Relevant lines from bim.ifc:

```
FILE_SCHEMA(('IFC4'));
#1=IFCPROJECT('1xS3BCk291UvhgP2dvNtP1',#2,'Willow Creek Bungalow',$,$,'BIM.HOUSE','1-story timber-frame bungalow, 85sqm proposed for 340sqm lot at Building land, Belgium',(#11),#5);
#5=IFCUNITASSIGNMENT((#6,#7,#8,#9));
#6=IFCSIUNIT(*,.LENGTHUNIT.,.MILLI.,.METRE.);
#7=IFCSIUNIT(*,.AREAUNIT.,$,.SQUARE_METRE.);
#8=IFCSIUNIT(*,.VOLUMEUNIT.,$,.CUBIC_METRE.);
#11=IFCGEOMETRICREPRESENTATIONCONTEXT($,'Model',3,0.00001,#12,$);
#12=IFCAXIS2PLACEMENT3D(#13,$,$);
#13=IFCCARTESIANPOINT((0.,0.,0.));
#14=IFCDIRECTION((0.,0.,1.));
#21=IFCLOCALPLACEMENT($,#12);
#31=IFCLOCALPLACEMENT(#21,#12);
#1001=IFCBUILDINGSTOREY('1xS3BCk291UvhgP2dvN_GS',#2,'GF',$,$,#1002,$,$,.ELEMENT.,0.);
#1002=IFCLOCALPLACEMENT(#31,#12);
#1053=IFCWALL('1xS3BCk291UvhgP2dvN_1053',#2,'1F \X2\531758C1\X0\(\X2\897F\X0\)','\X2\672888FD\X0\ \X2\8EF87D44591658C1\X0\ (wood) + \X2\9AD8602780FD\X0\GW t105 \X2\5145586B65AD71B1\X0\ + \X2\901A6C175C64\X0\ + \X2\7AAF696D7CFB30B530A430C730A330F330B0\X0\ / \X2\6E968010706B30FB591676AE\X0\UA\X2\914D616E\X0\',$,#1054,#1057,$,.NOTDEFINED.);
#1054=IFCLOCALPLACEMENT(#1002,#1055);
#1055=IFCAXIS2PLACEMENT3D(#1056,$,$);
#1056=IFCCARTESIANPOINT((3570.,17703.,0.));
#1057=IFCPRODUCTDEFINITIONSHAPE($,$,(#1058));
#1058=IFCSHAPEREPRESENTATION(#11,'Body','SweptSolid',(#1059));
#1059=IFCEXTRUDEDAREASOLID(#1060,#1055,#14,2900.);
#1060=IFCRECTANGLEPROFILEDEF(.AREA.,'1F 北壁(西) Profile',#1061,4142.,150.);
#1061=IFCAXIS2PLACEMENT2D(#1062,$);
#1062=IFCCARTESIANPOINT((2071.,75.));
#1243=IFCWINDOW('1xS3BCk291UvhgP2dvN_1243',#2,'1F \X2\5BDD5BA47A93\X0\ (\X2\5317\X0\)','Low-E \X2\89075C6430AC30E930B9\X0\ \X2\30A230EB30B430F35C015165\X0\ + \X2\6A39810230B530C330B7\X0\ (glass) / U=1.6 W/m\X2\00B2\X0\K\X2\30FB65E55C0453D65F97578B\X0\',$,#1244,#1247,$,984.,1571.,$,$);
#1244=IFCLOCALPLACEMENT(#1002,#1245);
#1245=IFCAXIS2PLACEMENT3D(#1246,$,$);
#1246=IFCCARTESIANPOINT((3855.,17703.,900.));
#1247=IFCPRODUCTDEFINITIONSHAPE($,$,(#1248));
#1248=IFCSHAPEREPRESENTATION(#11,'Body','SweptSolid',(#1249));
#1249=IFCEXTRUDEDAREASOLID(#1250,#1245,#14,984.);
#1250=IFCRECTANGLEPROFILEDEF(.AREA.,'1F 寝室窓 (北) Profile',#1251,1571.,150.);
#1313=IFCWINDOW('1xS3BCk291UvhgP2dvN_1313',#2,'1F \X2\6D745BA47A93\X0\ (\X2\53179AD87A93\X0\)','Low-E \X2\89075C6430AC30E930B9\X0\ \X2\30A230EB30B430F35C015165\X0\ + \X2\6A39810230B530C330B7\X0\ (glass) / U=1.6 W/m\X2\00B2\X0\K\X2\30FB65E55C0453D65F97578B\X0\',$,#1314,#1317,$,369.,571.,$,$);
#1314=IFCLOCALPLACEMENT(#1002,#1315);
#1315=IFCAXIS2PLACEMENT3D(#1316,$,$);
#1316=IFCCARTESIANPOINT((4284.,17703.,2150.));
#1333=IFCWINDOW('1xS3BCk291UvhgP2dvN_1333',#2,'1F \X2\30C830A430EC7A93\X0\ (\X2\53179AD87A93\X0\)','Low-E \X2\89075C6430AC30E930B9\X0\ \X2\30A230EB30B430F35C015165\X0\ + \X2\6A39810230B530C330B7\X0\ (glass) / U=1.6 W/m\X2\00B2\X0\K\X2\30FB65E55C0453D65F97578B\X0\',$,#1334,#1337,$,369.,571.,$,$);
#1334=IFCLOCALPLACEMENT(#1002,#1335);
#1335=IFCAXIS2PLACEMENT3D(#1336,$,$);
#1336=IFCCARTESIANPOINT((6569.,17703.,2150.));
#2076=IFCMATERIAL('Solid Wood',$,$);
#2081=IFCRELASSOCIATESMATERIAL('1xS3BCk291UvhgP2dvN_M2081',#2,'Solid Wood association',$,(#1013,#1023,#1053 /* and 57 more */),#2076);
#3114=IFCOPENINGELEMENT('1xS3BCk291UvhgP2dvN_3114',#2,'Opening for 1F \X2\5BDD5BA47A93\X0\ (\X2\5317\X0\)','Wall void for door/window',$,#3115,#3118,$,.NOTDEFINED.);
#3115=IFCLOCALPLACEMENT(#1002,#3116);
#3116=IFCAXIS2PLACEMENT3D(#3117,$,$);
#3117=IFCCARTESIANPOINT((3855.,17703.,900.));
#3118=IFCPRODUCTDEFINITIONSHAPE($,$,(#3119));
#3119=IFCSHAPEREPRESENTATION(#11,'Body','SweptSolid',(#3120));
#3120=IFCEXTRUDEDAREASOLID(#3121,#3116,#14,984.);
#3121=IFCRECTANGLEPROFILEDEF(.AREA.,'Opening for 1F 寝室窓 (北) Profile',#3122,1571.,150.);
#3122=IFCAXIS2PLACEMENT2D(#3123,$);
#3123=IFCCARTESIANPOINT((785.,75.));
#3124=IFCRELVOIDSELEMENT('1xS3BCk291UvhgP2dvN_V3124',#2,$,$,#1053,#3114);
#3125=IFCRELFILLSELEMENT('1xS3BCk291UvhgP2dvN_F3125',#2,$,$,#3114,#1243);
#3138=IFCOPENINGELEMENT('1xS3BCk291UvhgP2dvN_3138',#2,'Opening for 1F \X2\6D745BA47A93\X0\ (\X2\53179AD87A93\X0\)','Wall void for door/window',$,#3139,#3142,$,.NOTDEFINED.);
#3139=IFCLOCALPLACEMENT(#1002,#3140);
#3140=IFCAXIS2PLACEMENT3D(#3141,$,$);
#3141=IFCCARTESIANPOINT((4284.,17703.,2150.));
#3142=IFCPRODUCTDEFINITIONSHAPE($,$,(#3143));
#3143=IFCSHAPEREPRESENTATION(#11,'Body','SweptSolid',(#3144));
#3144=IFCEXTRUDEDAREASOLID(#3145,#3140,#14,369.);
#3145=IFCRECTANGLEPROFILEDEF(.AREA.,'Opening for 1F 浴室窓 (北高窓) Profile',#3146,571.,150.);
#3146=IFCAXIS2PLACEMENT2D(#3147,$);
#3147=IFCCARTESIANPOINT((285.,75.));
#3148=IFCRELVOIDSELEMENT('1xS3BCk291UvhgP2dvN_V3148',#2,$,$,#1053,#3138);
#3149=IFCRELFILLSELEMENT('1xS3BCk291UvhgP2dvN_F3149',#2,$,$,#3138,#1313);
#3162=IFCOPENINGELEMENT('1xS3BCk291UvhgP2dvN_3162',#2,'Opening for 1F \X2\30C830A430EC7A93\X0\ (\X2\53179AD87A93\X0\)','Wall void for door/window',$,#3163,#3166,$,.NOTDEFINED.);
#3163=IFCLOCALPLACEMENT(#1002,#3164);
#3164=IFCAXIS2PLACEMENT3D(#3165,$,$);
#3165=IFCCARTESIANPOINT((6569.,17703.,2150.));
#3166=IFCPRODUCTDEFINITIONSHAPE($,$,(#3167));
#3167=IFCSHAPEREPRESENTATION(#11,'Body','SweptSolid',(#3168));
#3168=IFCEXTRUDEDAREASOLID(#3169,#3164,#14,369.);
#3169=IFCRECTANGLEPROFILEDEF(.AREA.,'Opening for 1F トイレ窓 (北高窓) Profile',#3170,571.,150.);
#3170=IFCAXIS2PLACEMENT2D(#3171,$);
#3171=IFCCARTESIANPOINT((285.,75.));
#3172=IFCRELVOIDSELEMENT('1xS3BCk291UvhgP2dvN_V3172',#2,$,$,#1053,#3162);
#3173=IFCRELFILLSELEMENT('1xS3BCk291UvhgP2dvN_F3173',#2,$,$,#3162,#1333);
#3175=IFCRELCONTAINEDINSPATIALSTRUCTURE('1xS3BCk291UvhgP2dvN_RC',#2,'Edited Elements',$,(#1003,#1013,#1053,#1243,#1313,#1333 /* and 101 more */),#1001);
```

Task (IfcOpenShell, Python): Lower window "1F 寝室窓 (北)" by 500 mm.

```python
import numpy as np
import ifcopenshell
import ifcopenshell.api.geometry
import ifcopenshell.util.placement
import ifcopenshell.util.unit

model = ifcopenshell.open("bim.ifc")
unit_scale = ifcopenshell.util.unit.calculate_unit_scale(model)

window = model.by_id(1243)
opening = window.FillsVoids[0].RelatingOpeningElement
dz = -0.5 / unit_scale

shift = np.array([0.0, 0.0, dz])
# The window is not placed relative to its opening, so move both.
for product in (opening, window):
    matrix = ifcopenshell.util.placement.get_local_placement(product.ObjectPlacement)
    matrix[:3, 3] += shift
    ifcopenshell.api.geometry.edit_object_placement(model, product=product, matrix=matrix, is_si=False)

print(f"moved by {dz * unit_scale:+.3f} m")

model.write("bim_updated.ifc")
```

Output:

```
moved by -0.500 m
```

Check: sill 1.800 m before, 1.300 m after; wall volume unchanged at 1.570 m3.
